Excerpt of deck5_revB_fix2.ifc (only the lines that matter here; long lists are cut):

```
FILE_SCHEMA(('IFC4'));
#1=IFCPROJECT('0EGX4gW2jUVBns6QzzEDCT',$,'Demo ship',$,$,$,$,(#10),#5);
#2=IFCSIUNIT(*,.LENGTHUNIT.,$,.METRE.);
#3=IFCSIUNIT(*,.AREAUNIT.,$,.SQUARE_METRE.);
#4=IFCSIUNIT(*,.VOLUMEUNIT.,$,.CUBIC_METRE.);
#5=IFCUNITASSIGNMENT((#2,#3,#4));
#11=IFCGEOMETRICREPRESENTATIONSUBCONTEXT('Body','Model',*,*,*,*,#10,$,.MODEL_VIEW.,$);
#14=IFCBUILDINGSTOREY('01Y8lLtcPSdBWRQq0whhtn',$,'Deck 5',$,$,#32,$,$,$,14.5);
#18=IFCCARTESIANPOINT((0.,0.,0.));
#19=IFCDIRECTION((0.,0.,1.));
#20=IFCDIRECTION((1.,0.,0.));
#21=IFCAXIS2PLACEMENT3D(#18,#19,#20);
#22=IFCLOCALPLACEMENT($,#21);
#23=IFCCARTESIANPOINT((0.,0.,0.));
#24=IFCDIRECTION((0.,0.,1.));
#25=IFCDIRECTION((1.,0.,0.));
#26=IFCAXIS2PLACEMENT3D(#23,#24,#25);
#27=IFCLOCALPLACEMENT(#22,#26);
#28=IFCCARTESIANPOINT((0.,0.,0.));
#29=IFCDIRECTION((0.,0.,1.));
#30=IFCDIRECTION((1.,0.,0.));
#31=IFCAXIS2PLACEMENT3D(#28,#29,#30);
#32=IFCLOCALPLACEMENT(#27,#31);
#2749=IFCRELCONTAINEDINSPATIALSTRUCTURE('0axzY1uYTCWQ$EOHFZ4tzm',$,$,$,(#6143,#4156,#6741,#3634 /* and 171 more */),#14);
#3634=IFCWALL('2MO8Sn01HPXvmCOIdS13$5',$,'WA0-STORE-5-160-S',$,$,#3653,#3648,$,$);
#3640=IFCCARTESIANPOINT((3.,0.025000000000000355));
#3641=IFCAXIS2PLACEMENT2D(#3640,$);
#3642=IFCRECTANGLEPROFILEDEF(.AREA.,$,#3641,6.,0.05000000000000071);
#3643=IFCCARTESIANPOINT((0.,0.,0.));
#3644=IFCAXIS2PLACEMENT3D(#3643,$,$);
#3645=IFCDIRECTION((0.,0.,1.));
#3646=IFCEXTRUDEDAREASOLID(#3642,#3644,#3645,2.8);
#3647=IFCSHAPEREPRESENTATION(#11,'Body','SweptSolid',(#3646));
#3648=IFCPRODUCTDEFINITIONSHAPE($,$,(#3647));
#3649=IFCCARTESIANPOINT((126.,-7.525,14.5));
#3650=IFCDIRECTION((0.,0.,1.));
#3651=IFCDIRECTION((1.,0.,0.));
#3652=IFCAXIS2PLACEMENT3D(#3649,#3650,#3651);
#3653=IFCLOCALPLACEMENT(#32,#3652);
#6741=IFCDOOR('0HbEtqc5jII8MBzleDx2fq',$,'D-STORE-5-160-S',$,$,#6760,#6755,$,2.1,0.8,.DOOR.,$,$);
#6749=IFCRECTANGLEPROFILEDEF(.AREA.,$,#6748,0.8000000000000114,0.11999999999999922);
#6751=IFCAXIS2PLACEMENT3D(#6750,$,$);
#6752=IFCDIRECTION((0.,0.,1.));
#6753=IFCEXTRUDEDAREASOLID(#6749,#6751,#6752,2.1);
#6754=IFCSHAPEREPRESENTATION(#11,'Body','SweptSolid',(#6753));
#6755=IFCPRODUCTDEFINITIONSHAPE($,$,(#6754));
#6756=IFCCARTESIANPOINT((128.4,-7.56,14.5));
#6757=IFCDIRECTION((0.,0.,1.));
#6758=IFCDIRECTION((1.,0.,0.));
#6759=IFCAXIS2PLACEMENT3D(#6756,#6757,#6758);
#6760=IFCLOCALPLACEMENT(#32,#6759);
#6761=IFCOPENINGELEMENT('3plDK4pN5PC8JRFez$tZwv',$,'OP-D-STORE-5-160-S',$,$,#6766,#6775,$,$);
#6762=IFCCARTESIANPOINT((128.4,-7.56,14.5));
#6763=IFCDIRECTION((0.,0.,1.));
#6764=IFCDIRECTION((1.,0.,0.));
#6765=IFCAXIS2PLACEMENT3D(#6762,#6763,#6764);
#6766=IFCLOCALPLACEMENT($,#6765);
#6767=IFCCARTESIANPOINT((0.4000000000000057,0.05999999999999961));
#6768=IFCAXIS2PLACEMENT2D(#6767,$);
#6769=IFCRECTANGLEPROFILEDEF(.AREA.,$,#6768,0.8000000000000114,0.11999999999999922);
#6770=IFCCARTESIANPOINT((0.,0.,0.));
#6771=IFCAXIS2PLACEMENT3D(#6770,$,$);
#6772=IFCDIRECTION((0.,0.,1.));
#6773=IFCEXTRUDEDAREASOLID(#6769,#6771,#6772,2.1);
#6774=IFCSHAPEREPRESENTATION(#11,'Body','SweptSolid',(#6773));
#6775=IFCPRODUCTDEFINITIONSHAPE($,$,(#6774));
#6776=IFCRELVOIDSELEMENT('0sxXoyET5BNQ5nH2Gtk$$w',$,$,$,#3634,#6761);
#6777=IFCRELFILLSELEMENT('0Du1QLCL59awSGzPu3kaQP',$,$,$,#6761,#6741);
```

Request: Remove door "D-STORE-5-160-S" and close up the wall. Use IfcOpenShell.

```python
import ifcopenshell
import ifcopenshell.api.feature
import ifcopenshell.api.root
import ifcopenshell.geom
import ifcopenshell.util.shape

model = ifcopenshell.open("deck5_revB_fix2.ifc")
settings = ifcopenshell.geom.settings()


def volume(element):
    """Net volume in cubic metres, openings subtracted."""
    shape = ifcopenshell.geom.create_shape(settings, element)
    return ifcopenshell.util.shape.get_volume(shape.geometry)


door = model.by_id(6741)
opening = door.FillsVoids[0].RelatingOpeningElement
wall = opening.VoidsElements[0].RelatingBuildingElement
before = volume(wall)

ifcopenshell.api.root.remove_product(model, product=door)
ifcopenshell.api.feature.remove_feature(model, feature=opening)

after = volume(wall)

print(f"wall volume {before:.3f} -> {after:.3f} m3")

model.write("deck5_revB_fix2-out.ifc")
```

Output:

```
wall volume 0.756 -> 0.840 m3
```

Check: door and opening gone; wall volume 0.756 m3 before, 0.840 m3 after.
